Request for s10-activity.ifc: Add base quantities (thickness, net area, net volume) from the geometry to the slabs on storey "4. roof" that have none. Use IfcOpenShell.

First a look at what the model holds.

```python
import ifcopenshell
import ifcopenshell.util.element
import ifcopenshell.util.unit

model = ifcopenshell.open("s10-activity.ifc")
print(model.schema)
for unit_type in ("LENGTHUNIT", "AREAUNIT", "VOLUMEUNIT"):
    print(unit_type, ifcopenshell.util.unit.calculate_unit_scale(model, unit_type))
storey = next(s for s in model.by_type("IfcBuildingStorey") if s.Name == "4. roof")
slabs = [e for e in ifcopenshell.util.element.get_decomposition(storey) if e.is_a("IfcSlab")]
for e in sorted(slabs, key=lambda e: e.id()):
    print(e.id(), e.is_a(), e.Name, list(ifcopenshell.util.element.get_psets(e, qtos_only=True)), sep=" | ")
```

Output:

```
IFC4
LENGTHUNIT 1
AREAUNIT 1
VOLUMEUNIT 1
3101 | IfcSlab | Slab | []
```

```python
import ifcopenshell
import ifcopenshell.api.pset
import ifcopenshell.geom
import ifcopenshell.util.element
import ifcopenshell.util.shape
import ifcopenshell.util.unit

model = ifcopenshell.open("s10-activity.ifc")
unit_scale = ifcopenshell.util.unit.calculate_unit_scale(model)
area_scale = ifcopenshell.util.unit.calculate_unit_scale(model, "AREAUNIT")
volume_scale = ifcopenshell.util.unit.calculate_unit_scale(model, "VOLUMEUNIT")
settings = ifcopenshell.geom.settings()

storey = next(s for s in model.by_type("IfcBuildingStorey") if s.Name == "4. roof")
slabs = [e for e in ifcopenshell.util.element.get_decomposition(storey) if e.is_a("IfcSlab")]

for e in sorted(slabs, key=lambda e: e.id()):
    if ifcopenshell.util.element.get_psets(e, qtos_only=True, should_inherit=False):
        continue
    # Geometry comes back in metres, in the element's own axes.
    shape = ifcopenshell.geom.create_shape(settings, e)
    values = {
        "Width": ifcopenshell.util.shape.get_z(shape.geometry) / unit_scale,
        "NetArea": ifcopenshell.util.shape.get_footprint_area(shape.geometry) / area_scale,
        "NetVolume": ifcopenshell.util.shape.get_volume(shape.geometry) / volume_scale,
    }
    qto = ifcopenshell.api.pset.add_qto(model, product=e, name="Qto_SlabBaseQuantities")
    ifcopenshell.api.pset.edit_qto(model, qto=qto, properties=values)
    print(e.id(), {k: round(v, 3) for k, v in values.items()})

model.write("s10-activity_edited.ifc")
```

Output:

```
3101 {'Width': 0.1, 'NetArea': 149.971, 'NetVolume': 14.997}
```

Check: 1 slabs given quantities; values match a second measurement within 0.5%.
